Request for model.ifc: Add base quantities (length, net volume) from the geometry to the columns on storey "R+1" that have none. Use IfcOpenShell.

First a look at what the model holds.

```python
import ifcopenshell
import ifcopenshell.util.element
import ifcopenshell.util.unit

model = ifcopenshell.open("model.ifc")
print(model.schema)
for unit_type in ("LENGTHUNIT", "AREAUNIT", "VOLUMEUNIT"):
    print(unit_type, ifcopenshell.util.unit.calculate_unit_scale(model, unit_type))
storey = next(s for s in model.by_type("IfcBuildingStorey") if s.Name == "R+1")
columns = [e for e in ifcopenshell.util.element.get_decomposition(storey) if e.is_a("IfcColumn")]
for e in sorted(columns, key=lambda e: e.id()):
    print(e.id(), e.is_a(), e.Name, list(ifcopenshell.util.element.get_psets(e, qtos_only=True)), sep=" | ")
```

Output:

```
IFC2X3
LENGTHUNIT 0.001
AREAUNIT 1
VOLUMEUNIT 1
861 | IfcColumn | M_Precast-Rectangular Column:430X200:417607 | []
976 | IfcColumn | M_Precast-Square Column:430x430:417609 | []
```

```python
import ifcopenshell
import ifcopenshell.api.pset
import ifcopenshell.geom
import ifcopenshell.util.element
import ifcopenshell.util.shape
import ifcopenshell.util.unit

model = ifcopenshell.open("model.ifc")
unit_scale = ifcopenshell.util.unit.calculate_unit_scale(model)
volume_scale = ifcopenshell.util.unit.calculate_unit_scale(model, "VOLUMEUNIT")
settings = ifcopenshell.geom.settings()

storey = next(s for s in model.by_type("IfcBuildingStorey") if s.Name == "R+1")
columns = [e for e in ifcopenshell.util.element.get_decomposition(storey) if e.is_a("IfcColumn")]

for e in sorted(columns, key=lambda e: e.id()):
    if ifcopenshell.util.element.get_psets(e, qtos_only=True, should_inherit=False):
        continue
    # Geometry comes back in metres, in the element's own axes.
    shape = ifcopenshell.geom.create_shape(settings, e)
    values = {
        "Length": ifcopenshell.util.shape.get_z(shape.geometry) / unit_scale,
        "NetVolume": ifcopenshell.util.shape.get_volume(shape.geometry) / volume_scale,
    }
    qto = ifcopenshell.api.pset.add_qto(model, product=e, name="BaseQuantities")
    ifcopenshell.api.pset.edit_qto(model, qto=qto, properties=values)
    print(e.id(), {k: round(v, 3) for k, v in values.items()})

model.write("model-out.ifc")
```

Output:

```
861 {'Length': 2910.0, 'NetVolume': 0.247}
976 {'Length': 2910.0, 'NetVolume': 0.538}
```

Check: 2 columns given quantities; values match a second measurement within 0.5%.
